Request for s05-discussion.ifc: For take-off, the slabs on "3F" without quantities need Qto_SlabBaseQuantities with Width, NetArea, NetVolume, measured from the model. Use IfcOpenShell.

First a look at what the model holds.

```python
import ifcopenshell
import ifcopenshell.util.element
import ifcopenshell.util.unit

model = ifcopenshell.open("s05-discussion.ifc")
print(model.schema)
for unit_type in ("LENGTHUNIT", "AREAUNIT", "VOLUMEUNIT"):
    print(unit_type, ifcopenshell.util.unit.calculate_unit_scale(model, unit_type))
storey = next(s for s in model.by_type("IfcBuildingStorey") if s.Name == "3F")
slabs = [e for e in ifcopenshell.util.element.get_decomposition(storey) if e.is_a("IfcSlab")]
for e in sorted(slabs, key=lambda e: e.id()):
    print(e.id(), e.is_a(), e.Name, list(ifcopenshell.util.element.get_psets(e, qtos_only=True)), sep=" | ")
```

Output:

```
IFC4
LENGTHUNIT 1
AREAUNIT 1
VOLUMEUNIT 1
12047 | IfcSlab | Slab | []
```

```python
import ifcopenshell
import ifcopenshell.api.pset
import ifcopenshell.geom
import ifcopenshell.util.element
import ifcopenshell.util.shape
import ifcopenshell.util.unit

model = ifcopenshell.open("s05-discussion.ifc")
unit_scale = ifcopenshell.util.unit.calculate_unit_scale(model)
area_scale = ifcopenshell.util.unit.calculate_unit_scale(model, "AREAUNIT")
volume_scale = ifcopenshell.util.unit.calculate_unit_scale(model, "VOLUMEUNIT")
settings = ifcopenshell.geom.settings()

storey = next(s for s in model.by_type("IfcBuildingStorey") if s.Name == "3F")
slabs = [e for e in ifcopenshell.util.element.get_decomposition(storey) if e.is_a("IfcSlab")]

for e in sorted(slabs, key=lambda e: e.id()):
    if ifcopenshell.util.element.get_psets(e, qtos_only=True, should_inherit=False):
        continue
    # Geometry comes back in metres, in the element's own axes.
    shape = ifcopenshell.geom.create_shape(settings, e)
    values = {
        "Width": ifcopenshell.util.shape.get_z(shape.geometry) / unit_scale,
        "NetArea": ifcopenshell.util.shape.get_footprint_area(shape.geometry) / area_scale,
        "NetVolume": ifcopenshell.util.shape.get_volume(shape.geometry) / volume_scale,
    }
    qto = ifcopenshell.api.pset.add_qto(model, product=e, name="Qto_SlabBaseQuantities")
    ifcopenshell.api.pset.edit_qto(model, qto=qto, properties=values)
    print(e.id(), {k: round(v, 3) for k, v in values.items()})

model.write("s05-discussion_edited.ifc")
```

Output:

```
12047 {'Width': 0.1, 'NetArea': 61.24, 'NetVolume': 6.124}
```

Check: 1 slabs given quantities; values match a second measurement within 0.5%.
